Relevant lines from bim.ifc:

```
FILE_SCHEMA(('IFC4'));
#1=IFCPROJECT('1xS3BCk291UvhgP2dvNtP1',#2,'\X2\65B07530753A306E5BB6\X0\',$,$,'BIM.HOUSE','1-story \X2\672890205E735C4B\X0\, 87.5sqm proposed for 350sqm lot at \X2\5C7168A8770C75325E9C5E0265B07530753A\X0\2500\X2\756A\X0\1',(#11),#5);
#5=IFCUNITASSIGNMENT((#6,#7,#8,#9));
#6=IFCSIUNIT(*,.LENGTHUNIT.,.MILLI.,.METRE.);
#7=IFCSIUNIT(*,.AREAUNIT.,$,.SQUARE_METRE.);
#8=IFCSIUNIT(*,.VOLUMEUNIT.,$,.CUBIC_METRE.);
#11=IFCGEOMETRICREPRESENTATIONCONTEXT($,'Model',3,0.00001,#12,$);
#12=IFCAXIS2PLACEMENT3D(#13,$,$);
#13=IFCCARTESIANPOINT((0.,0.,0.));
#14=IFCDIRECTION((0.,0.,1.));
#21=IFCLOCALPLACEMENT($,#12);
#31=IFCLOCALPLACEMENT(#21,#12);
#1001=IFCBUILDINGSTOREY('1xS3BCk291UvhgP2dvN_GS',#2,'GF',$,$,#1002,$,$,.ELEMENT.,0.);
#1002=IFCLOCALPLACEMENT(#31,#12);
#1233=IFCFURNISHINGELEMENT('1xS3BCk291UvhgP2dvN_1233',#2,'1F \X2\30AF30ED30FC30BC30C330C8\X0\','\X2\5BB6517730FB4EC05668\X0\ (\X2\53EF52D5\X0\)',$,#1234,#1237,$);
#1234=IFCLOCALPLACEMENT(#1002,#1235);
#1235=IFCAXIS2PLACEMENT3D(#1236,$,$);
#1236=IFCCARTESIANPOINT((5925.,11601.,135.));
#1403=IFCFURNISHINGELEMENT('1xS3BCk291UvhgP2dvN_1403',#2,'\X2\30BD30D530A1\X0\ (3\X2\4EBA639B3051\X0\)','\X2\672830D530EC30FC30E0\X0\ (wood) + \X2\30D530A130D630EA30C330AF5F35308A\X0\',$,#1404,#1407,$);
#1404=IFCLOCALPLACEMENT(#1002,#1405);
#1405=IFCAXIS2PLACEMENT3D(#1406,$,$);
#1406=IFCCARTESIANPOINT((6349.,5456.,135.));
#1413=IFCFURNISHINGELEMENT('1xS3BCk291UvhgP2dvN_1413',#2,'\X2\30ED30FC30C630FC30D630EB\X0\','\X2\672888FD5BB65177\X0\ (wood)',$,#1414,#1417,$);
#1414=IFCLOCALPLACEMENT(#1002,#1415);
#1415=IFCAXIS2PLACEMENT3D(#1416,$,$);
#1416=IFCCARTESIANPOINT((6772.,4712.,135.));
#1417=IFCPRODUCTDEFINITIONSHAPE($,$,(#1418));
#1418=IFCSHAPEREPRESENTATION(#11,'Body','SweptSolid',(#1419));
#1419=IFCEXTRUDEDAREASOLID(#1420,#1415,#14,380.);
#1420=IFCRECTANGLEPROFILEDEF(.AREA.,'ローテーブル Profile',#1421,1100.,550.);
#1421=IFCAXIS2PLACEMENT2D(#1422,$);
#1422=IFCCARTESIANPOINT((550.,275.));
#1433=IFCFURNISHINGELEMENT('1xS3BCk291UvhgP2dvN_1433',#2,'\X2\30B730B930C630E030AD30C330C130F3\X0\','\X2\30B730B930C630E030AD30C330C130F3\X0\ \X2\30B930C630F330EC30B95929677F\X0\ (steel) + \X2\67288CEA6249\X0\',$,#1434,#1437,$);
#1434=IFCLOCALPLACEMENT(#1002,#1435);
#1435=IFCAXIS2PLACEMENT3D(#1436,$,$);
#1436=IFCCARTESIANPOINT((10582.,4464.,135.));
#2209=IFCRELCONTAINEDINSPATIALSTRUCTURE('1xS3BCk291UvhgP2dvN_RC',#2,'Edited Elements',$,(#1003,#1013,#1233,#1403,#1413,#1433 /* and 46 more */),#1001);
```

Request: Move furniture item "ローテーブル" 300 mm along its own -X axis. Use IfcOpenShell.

```python
import ifcopenshell
import ifcopenshell.api.geometry
import ifcopenshell.util.placement
import ifcopenshell.util.unit

model = ifcopenshell.open("bim.ifc")
unit_scale = ifcopenshell.util.unit.calculate_unit_scale(model)

item = model.by_id(1413)
matrix = ifcopenshell.util.placement.get_local_placement(item.ObjectPlacement)
matrix[:3, 3] -= matrix[:3, 0] * 0.3 / unit_scale
ifcopenshell.api.geometry.edit_object_placement(model, product=item, matrix=matrix, is_si=False)

print(ifcopenshell.util.placement.get_local_placement(item.ObjectPlacement).round(3) + 0.0)

model.write("bim-out.ifc")
```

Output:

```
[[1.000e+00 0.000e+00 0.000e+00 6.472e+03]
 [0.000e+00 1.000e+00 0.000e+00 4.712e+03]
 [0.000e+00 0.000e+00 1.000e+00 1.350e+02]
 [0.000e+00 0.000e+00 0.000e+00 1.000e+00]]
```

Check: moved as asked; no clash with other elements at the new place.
